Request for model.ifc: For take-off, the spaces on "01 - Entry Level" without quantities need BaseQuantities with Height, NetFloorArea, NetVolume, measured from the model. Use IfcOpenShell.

First a look at what the model holds.

```python
import ifcopenshell
import ifcopenshell.util.element
import ifcopenshell.util.unit

model = ifcopenshell.open("model.ifc")
print(model.schema)
for unit_type in ("LENGTHUNIT", "AREAUNIT", "VOLUMEUNIT"):
    print(unit_type, ifcopenshell.util.unit.calculate_unit_scale(model, unit_type))
storey = next(s for s in model.by_type("IfcBuildingStorey") if s.Name == "01 - Entry Level")
spaces = [e for e in ifcopenshell.util.element.get_decomposition(storey) if e.is_a("IfcSpace")]
for e in sorted(spaces, key=lambda e: e.id()):
    print(e.id(), e.is_a(), e.Name, list(ifcopenshell.util.element.get_psets(e, qtos_only=True)), sep=" | ")
```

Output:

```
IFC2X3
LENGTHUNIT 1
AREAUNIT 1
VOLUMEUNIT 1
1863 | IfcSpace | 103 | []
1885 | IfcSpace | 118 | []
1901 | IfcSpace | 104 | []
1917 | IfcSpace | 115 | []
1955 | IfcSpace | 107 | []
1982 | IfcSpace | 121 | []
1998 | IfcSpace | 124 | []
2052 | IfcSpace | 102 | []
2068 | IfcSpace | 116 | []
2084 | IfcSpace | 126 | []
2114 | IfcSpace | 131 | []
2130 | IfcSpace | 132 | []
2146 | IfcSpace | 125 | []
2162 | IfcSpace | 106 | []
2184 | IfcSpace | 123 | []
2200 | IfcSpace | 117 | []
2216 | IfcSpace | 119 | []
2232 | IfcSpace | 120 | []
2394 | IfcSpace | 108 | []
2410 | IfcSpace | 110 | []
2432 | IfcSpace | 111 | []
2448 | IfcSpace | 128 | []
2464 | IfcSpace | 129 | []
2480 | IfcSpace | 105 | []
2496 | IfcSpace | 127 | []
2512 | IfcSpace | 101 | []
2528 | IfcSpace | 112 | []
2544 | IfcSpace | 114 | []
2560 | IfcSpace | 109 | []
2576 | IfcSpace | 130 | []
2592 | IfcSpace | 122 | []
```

```python
import ifcopenshell
import ifcopenshell.api.pset
import ifcopenshell.geom
import ifcopenshell.util.element
import ifcopenshell.util.shape
import ifcopenshell.util.unit

model = ifcopenshell.open("model.ifc")
unit_scale = ifcopenshell.util.unit.calculate_unit_scale(model)
area_scale = ifcopenshell.util.unit.calculate_unit_scale(model, "AREAUNIT")
volume_scale = ifcopenshell.util.unit.calculate_unit_scale(model, "VOLUMEUNIT")
settings = ifcopenshell.geom.settings()

storey = next(s for s in model.by_type("IfcBuildingStorey") if s.Name == "01 - Entry Level")
spaces = [e for e in ifcopenshell.util.element.get_decomposition(storey) if e.is_a("IfcSpace")]

for e in sorted(spaces, key=lambda e: e.id()):
    if ifcopenshell.util.element.get_psets(e, qtos_only=True, should_inherit=False):
        continue
    # Geometry comes back in metres, in the element's own axes.
    shape = ifcopenshell.geom.create_shape(settings, e)
    values = {
        "Height": ifcopenshell.util.shape.get_z(shape.geometry) / unit_scale,
        "NetFloorArea": ifcopenshell.util.shape.get_footprint_area(shape.geometry) / area_scale,
        "NetVolume": ifcopenshell.util.shape.get_volume(shape.geometry) / volume_scale,
    }
    qto = ifcopenshell.api.pset.add_qto(model, product=e, name="BaseQuantities")
    ifcopenshell.api.pset.edit_qto(model, qto=qto, properties=values)
    print(e.id(), {k: round(v, 3) for k, v in values.items()})

model.write("model_edited.ifc")
```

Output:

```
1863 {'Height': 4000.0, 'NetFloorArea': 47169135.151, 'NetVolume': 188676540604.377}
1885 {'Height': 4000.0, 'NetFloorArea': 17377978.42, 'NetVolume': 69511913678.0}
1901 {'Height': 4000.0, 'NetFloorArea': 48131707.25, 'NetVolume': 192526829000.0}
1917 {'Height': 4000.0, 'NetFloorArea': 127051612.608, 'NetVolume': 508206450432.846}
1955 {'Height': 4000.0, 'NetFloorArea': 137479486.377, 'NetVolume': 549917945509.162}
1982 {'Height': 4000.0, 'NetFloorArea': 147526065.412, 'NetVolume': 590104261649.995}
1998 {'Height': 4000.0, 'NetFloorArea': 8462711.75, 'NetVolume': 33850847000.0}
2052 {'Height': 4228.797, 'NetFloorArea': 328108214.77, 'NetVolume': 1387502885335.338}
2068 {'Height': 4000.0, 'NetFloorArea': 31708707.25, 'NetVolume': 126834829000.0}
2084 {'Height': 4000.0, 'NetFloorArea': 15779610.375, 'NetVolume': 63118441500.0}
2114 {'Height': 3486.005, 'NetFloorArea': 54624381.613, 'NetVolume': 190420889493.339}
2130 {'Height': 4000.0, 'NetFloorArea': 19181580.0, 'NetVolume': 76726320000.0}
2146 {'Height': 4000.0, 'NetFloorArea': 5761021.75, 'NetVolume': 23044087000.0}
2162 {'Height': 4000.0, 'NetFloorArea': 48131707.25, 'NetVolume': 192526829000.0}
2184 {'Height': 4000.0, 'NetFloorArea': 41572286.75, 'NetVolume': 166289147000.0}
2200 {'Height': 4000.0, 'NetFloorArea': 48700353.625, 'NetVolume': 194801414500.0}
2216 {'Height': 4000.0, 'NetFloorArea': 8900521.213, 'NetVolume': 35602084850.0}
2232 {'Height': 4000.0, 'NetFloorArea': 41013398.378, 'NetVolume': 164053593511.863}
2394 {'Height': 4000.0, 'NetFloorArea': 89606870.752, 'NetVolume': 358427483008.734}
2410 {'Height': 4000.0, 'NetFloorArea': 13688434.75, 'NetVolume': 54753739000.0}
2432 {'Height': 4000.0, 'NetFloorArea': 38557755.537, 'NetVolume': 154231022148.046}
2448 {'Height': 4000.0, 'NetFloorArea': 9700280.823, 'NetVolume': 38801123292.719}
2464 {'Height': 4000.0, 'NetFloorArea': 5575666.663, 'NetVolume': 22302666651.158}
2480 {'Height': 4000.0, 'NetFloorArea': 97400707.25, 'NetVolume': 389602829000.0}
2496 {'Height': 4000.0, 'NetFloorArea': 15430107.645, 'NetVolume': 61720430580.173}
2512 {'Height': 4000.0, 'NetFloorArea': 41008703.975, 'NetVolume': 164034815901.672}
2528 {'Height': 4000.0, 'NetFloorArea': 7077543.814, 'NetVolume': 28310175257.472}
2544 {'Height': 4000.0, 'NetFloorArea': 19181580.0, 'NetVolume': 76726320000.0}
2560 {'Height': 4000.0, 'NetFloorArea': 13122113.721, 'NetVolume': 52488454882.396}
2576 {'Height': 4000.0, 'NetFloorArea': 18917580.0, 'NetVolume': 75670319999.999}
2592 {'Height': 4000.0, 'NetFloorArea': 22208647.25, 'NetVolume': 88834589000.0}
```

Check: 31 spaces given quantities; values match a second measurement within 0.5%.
